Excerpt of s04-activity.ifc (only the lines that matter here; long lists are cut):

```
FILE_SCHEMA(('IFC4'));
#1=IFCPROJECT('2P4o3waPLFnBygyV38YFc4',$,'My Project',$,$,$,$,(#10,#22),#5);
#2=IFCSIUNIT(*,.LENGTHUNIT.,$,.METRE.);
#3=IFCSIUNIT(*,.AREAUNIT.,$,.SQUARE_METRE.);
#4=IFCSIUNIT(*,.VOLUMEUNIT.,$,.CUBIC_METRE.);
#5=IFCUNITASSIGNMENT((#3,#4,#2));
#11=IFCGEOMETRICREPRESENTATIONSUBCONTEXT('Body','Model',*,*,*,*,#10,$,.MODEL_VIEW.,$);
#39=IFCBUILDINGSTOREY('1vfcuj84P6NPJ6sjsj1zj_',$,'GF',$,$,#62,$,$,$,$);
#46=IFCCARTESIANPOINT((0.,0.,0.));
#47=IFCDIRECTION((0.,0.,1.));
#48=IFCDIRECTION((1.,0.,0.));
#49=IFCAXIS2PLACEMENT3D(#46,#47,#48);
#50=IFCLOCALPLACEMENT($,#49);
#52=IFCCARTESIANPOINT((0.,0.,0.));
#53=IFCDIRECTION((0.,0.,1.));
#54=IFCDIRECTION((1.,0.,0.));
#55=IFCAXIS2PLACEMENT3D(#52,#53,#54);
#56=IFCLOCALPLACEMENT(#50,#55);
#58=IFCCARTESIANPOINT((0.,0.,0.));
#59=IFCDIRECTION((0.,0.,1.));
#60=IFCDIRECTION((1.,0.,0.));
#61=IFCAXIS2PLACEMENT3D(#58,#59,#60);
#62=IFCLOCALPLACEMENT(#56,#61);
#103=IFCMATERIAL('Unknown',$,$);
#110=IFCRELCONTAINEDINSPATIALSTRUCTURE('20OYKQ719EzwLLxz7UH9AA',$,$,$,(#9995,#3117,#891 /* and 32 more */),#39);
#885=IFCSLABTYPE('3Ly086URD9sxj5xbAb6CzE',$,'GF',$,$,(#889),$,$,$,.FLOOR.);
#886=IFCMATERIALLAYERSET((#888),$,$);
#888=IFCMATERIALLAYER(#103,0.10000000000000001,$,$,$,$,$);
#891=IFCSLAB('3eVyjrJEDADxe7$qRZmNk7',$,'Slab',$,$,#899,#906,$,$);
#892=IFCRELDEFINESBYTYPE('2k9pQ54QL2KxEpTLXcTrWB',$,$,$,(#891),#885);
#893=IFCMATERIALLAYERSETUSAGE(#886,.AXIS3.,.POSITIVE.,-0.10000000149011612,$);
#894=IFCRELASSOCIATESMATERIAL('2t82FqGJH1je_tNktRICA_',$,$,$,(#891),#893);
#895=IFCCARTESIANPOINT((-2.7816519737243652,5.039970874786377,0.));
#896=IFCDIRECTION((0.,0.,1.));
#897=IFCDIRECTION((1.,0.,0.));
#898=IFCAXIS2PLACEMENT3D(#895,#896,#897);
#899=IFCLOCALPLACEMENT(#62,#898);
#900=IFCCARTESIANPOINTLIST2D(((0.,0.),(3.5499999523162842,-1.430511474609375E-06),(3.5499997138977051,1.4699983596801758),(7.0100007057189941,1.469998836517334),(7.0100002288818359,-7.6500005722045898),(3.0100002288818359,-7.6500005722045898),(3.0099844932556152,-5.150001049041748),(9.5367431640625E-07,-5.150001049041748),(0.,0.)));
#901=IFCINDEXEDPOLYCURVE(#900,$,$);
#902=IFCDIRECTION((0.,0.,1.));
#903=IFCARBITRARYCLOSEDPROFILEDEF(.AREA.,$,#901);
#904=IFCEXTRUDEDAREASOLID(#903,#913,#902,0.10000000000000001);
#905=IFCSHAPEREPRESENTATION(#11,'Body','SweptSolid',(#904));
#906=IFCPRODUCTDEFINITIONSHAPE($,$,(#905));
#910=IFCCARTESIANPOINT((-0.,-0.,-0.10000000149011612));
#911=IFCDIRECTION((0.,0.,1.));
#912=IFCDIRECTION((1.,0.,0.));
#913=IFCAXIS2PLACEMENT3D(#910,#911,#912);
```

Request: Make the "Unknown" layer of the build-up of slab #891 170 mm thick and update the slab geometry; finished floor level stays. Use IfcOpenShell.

```python
import ifcopenshell
import ifcopenshell.util.element
import ifcopenshell.util.representation
import ifcopenshell.util.unit

model = ifcopenshell.open("s04-activity.ifc")
unit_scale = ifcopenshell.util.unit.calculate_unit_scale(model)

layer_set = model.by_id(886)
layer = next(l for l in layer_set.MaterialLayers if l.Material and l.Material.Name == "Unknown")
change = 0.17 / unit_scale - layer.LayerThickness
layer.LayerThickness += change

# Geometry does not follow the layer set by itself.
slabs = [e for e in ifcopenshell.util.element.get_elements_by_material(model, layer_set) if e.is_a("IfcSlab")]
for slab in sorted(slabs, key=lambda e: e.id()):
    body = ifcopenshell.util.representation.get_representation(slab, "Model", "Body")
    solid = body.Items[0]
    old_depth = solid.Depth
    solid.Depth += change
    # Extruded upwards: lower the start of the extrusion so the top stays.
    x, y, z = solid.Position.Location.Coordinates
    solid.Position.Location = model.createIfcCartesianPoint((x, y, z - change))
    print(slab.id(), f"{old_depth:g} -> {solid.Depth:g}")

# The layers are counted up from the underside, which has moved.
for usage in {ifcopenshell.util.element.get_material(slab) for slab in slabs}:
    usage.OffsetFromReferenceLine -= change

model.write("s04-activity-out.ifc")
```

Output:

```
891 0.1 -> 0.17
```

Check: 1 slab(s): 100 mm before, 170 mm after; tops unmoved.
